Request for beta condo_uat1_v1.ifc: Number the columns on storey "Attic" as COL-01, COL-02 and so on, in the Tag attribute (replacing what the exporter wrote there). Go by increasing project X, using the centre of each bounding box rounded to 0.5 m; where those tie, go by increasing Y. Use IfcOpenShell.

First a look at what the model holds.

```python
import ifcopenshell
import ifcopenshell.util.element
import ifcopenshell.util.placement

model = ifcopenshell.open("beta condo_uat1_v1.ifc")
print(model.schema)
storey = next(s for s in model.by_type("IfcBuildingStorey") if s.Name == "Attic")
columns = [e for e in ifcopenshell.util.element.get_decomposition(storey) if e.is_a("IfcColumn")]
for e in sorted(columns, key=lambda e: e.id()):
    origin = ifcopenshell.util.placement.get_local_placement(e.ObjectPlacement)[:3, 3]
    print(e.id(), e.Tag, e.Name, origin.round(2) + 0.0, sep=" | ")
```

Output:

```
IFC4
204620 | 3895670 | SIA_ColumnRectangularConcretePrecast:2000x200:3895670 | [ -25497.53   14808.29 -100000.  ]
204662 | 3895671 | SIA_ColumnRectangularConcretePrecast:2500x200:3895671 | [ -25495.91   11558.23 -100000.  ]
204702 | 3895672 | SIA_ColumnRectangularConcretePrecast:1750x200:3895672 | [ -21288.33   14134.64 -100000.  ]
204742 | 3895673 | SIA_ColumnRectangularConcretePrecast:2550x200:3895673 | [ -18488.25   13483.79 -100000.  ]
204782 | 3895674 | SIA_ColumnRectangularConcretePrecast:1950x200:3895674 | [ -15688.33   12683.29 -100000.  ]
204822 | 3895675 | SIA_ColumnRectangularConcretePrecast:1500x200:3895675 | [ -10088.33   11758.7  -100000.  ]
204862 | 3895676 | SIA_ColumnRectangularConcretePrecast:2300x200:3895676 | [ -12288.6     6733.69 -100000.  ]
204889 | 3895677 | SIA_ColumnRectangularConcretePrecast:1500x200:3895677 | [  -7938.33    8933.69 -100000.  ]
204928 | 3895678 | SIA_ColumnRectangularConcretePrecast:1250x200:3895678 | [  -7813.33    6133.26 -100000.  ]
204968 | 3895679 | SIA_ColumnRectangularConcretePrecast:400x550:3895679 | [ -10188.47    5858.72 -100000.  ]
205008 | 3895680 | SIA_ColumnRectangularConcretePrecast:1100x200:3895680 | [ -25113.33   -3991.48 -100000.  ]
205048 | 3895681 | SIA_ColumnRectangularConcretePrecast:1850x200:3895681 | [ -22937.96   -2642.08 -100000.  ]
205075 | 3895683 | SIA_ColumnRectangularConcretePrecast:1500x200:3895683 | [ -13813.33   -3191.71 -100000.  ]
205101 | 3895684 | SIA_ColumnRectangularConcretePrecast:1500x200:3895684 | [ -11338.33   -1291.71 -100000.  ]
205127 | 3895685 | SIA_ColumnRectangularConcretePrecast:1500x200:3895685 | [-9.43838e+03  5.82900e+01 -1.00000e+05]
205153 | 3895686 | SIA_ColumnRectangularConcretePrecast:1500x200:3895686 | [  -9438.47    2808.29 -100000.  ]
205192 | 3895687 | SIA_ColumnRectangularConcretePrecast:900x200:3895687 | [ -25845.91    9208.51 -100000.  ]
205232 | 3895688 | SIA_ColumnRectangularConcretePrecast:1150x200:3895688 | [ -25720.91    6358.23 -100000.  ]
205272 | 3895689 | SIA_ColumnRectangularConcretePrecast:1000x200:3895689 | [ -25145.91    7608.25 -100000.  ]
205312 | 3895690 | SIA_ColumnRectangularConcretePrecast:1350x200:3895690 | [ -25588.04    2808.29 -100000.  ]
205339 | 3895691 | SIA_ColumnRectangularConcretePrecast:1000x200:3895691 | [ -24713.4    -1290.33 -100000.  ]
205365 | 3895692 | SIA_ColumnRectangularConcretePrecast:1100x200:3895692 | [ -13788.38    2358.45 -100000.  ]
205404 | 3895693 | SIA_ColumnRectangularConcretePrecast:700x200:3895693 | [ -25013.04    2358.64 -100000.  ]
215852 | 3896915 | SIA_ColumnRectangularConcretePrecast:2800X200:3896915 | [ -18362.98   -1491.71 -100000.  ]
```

```python
import ifcopenshell
import ifcopenshell.geom
import ifcopenshell.util.element
import ifcopenshell.util.shape

model = ifcopenshell.open("beta condo_uat1_v1.ifc")
settings = ifcopenshell.geom.settings()
settings.set("use-world-coords", True)


def centre(element):
    shape = ifcopenshell.geom.create_shape(settings, element)
    return ifcopenshell.util.shape.get_bbox_centroid(shape.geometry)


storey = next(s for s in model.by_type("IfcBuildingStorey") if s.Name == "Attic")
columns = [e for e in ifcopenshell.util.element.get_decomposition(storey) if e.is_a("IfcColumn")]

# Insertion points can sit at a corner or the storey origin, so sort by the geometry (in metres).
centres = {e: centre(e) for e in columns}
columns.sort(key=lambda e: (round(centres[e][0] / 0.5), centres[e][1]))

for i, e in enumerate(columns, start=1):
    number = f"COL-{i:02d}"
    e.Tag = number
    print(e.id(), number)

model.write("beta condo_uat1_v1_updated.ifc")
```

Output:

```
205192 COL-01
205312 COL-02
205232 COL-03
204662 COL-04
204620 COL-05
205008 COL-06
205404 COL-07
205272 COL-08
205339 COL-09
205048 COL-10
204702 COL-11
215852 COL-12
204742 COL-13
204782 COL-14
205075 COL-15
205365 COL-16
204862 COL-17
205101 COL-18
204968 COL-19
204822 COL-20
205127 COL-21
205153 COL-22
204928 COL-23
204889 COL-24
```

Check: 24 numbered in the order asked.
